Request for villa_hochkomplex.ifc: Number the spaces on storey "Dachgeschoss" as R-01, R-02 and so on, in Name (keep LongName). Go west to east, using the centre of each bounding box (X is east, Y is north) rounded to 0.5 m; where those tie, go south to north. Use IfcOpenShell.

First a look at what the model holds.

```python
import ifcopenshell
import ifcopenshell.util.element
import ifcopenshell.util.placement

model = ifcopenshell.open("villa_hochkomplex.ifc")
print(model.schema)
storey = next(s for s in model.by_type("IfcBuildingStorey") if s.Name == "Dachgeschoss")
spaces = [e for e in ifcopenshell.util.element.get_decomposition(storey) if e.is_a("IfcSpace")]
for e in sorted(spaces, key=lambda e: e.id()):
    origin = ifcopenshell.util.placement.get_local_placement(e.ObjectPlacement)[:3, 3]
    print(e.id(), e.Name, e.LongName, origin.round(2) + 0.0, sep=" | ")
```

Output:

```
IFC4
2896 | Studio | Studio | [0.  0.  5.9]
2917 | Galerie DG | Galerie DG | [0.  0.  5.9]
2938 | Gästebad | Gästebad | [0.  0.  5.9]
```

```python
import ifcopenshell
import ifcopenshell.geom
import ifcopenshell.util.element
import ifcopenshell.util.shape

model = ifcopenshell.open("villa_hochkomplex.ifc")
settings = ifcopenshell.geom.settings()
settings.set("use-world-coords", True)


def centre(element):
    shape = ifcopenshell.geom.create_shape(settings, element)
    return ifcopenshell.util.shape.get_bbox_centroid(shape.geometry)


storey = next(s for s in model.by_type("IfcBuildingStorey") if s.Name == "Dachgeschoss")
spaces = [e for e in ifcopenshell.util.element.get_decomposition(storey) if e.is_a("IfcSpace")]

# Insertion points can sit at a corner or the storey origin, so sort by the geometry (in metres).
centres = {e: centre(e) for e in spaces}
spaces.sort(key=lambda e: (round(centres[e][0] / 0.5), centres[e][1]))

for i, e in enumerate(spaces, start=1):
    number = f"R-{i:02d}"
    e.Name = number
    print(e.id(), number)

model.write("villa_hochkomplex_v2.ifc")
```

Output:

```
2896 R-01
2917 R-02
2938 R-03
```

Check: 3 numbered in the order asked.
